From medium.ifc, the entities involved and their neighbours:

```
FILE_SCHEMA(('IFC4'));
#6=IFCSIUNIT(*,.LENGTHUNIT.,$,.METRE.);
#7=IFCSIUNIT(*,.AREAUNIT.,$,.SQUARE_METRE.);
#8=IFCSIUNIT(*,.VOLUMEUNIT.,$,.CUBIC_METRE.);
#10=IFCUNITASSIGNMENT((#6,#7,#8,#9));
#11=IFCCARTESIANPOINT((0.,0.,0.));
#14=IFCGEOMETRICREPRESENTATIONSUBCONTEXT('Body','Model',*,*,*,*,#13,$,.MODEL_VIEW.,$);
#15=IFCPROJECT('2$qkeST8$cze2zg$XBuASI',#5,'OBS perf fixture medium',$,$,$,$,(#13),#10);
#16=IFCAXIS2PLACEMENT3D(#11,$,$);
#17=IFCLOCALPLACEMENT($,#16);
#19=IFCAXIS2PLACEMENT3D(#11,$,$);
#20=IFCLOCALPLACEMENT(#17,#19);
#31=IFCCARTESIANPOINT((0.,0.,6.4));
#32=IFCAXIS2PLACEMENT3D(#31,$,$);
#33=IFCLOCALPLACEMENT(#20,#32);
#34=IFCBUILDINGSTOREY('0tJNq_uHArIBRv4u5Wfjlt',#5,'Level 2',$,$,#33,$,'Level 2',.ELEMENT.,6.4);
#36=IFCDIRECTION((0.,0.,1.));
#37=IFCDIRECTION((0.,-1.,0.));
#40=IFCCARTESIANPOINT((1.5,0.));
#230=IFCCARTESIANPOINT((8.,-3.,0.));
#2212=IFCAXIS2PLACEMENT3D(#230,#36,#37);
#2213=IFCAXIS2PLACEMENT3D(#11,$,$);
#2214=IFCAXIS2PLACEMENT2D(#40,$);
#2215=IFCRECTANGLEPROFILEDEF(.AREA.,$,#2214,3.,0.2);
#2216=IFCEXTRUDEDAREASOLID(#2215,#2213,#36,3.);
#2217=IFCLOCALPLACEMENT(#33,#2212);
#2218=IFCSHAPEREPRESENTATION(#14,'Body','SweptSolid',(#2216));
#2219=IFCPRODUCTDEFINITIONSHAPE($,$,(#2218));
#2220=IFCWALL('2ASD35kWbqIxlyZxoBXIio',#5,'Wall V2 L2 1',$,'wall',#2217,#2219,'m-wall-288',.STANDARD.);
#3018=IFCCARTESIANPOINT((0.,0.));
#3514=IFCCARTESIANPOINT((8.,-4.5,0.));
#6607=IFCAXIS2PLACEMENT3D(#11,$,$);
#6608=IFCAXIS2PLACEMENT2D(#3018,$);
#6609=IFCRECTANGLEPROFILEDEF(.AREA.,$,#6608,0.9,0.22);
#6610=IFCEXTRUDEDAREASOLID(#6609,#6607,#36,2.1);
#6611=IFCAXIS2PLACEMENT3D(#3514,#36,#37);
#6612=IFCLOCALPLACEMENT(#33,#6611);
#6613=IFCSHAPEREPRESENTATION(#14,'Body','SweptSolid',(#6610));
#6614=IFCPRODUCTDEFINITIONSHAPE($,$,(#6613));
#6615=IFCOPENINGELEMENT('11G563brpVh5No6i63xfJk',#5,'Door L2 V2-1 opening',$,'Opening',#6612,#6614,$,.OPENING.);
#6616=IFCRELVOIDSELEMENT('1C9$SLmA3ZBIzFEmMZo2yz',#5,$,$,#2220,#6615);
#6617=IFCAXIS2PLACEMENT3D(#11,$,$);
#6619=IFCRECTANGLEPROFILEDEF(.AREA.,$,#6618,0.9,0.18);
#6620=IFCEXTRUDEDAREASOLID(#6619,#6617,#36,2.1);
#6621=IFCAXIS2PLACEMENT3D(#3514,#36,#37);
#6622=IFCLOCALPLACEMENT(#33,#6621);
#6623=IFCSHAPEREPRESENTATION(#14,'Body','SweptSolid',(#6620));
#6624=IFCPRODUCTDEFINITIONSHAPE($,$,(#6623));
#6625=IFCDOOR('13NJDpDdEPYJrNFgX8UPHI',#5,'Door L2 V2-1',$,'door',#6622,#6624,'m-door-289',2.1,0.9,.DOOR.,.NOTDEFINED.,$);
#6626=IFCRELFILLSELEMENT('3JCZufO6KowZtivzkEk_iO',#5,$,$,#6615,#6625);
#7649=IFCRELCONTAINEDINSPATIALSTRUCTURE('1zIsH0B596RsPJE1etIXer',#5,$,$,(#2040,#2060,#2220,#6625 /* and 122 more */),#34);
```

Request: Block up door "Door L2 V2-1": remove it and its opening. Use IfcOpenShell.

```python
import ifcopenshell
import ifcopenshell.api.feature
import ifcopenshell.api.root
import ifcopenshell.geom
import ifcopenshell.util.shape

model = ifcopenshell.open("medium.ifc")
settings = ifcopenshell.geom.settings()


def volume(element):
    """Net volume in cubic metres, openings subtracted."""
    shape = ifcopenshell.geom.create_shape(settings, element)
    return ifcopenshell.util.shape.get_volume(shape.geometry)


door = model.by_guid("13NJDpDdEPYJrNFgX8UPHI")
opening = door.FillsVoids[0].RelatingOpeningElement
wall = opening.VoidsElements[0].RelatingBuildingElement
before = volume(wall)

ifcopenshell.api.root.remove_product(model, product=door)
ifcopenshell.api.feature.remove_feature(model, feature=opening)

after = volume(wall)

print(f"wall volume {before:.3f} -> {after:.3f} m3")

model.write("medium-out.ifc")
```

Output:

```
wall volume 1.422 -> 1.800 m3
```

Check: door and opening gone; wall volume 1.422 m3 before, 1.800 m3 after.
